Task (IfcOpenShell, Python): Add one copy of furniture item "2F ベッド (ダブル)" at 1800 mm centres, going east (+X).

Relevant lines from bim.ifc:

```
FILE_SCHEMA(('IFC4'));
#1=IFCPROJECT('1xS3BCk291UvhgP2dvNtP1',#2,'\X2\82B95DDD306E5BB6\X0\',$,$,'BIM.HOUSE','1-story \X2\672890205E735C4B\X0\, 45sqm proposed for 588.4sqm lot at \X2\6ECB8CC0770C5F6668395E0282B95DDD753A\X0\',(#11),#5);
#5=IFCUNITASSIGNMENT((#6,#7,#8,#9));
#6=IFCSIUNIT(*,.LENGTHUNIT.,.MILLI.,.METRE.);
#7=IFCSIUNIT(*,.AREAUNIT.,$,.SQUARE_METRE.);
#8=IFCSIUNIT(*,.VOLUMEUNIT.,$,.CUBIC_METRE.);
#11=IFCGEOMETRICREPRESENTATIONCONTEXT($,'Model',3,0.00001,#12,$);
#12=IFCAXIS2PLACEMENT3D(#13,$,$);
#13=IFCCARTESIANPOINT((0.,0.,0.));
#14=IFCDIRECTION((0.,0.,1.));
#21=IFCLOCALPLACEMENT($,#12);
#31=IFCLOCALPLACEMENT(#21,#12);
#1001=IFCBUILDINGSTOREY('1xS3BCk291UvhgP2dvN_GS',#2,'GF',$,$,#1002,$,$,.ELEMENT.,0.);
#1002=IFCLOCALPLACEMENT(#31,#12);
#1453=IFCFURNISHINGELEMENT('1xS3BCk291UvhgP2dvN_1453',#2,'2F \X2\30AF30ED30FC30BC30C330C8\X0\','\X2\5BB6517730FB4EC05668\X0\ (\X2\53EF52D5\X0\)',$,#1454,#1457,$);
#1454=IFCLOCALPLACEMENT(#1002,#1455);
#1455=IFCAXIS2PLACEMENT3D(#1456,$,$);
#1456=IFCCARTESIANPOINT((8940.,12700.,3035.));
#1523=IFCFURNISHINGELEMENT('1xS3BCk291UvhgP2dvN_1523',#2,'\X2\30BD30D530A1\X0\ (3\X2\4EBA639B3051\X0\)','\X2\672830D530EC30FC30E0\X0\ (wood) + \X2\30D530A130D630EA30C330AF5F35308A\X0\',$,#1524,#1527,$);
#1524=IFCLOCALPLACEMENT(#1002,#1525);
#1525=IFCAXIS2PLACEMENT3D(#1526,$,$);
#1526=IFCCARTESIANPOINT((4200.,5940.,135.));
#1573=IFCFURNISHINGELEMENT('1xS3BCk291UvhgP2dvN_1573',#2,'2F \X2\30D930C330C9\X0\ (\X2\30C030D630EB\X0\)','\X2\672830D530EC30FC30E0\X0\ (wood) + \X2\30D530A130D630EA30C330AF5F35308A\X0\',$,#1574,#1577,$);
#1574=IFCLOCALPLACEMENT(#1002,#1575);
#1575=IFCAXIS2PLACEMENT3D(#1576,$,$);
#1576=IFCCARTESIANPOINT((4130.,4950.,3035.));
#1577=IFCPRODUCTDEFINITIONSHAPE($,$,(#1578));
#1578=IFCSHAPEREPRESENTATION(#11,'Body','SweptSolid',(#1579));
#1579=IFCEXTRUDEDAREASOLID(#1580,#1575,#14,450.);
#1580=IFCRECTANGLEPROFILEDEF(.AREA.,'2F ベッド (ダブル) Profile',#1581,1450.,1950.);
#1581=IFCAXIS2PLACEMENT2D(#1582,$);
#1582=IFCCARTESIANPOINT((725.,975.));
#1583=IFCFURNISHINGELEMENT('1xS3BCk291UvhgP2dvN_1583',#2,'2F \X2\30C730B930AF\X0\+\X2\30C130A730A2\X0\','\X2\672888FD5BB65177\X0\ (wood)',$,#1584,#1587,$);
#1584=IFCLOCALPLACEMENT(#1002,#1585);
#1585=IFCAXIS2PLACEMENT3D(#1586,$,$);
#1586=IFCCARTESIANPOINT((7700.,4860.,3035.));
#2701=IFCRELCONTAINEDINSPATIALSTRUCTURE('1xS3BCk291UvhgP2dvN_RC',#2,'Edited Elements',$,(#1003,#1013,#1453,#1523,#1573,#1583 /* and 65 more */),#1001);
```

```python
import numpy as np
import ifcopenshell
import ifcopenshell.api.geometry
import ifcopenshell.api.root
import ifcopenshell.util.element
import ifcopenshell.util.placement

model = ifcopenshell.open("bim.ifc")


def reuse_history(source, copy):
    """copy_class also copies each property set's owner history, people and application; keep the originals."""
    for rel in copy.IsDefinedBy:
        if rel.is_a("IfcRelDefinesByProperties") and (history := rel.RelatingPropertyDefinition.OwnerHistory):
            rel.RelatingPropertyDefinition.OwnerHistory = source.OwnerHistory
            ifcopenshell.util.element.remove_deep2(model, history)


source = model.by_guid("1xS3BCk291UvhgP2dvN_1573")
base = ifcopenshell.util.placement.get_local_placement(source.ObjectPlacement)
step = np.array([1.0, 0.0, 0.0]) * 1800.0

for i in range(1, 2):
    copy = ifcopenshell.api.root.copy_class(model, product=source)
    copy.Representation = ifcopenshell.util.element.copy_deep(
        model, source.Representation, exclude=["IfcGeometricRepresentationContext", "IfcRepresentationMap"]
    )
    reuse_history(source, copy)
    matrix = base.copy()
    matrix[:3, 3] += i * step
    print("added at", matrix[:3, 3].round(3) + 0.0)
    ifcopenshell.api.geometry.edit_object_placement(model, product=copy, matrix=matrix, is_si=False)

model.write("bim_v2.ifc")
```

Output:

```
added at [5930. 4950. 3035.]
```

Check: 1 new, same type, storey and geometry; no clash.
